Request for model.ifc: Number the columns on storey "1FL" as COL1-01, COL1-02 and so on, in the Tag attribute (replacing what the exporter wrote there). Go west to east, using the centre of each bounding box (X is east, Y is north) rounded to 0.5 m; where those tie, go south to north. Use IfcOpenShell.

First a look at what the model holds.

```python
import ifcopenshell
import ifcopenshell.util.element
import ifcopenshell.util.placement

model = ifcopenshell.open("model.ifc")
print(model.schema)
storey = next(s for s in model.by_type("IfcBuildingStorey") if s.Name == "1FL")
columns = [e for e in ifcopenshell.util.element.get_decomposition(storey) if e.is_a("IfcColumn")]
for e in sorted(columns, key=lambda e: e.id()):
    origin = ifcopenshell.util.placement.get_local_placement(e.ObjectPlacement)[:3, 3]
    print(e.id(), e.Tag, e.Name, origin.round(2) + 0.0, sep=" | ")
```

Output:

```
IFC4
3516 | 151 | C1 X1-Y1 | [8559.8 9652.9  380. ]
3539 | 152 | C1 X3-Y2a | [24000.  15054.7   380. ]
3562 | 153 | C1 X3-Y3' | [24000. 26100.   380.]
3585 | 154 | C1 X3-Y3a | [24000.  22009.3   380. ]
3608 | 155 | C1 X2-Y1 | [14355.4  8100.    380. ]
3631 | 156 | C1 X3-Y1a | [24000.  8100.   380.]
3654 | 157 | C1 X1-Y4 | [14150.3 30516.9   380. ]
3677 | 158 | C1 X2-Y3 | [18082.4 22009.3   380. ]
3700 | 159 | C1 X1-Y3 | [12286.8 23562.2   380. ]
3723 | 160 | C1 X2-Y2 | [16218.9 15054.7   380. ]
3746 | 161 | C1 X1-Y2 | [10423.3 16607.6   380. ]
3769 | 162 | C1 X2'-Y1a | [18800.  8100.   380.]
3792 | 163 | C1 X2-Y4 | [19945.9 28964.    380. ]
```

```python
import ifcopenshell
import ifcopenshell.geom
import ifcopenshell.util.element
import ifcopenshell.util.shape

model = ifcopenshell.open("model.ifc")
settings = ifcopenshell.geom.settings()
settings.set("use-world-coords", True)


def centre(element):
    shape = ifcopenshell.geom.create_shape(settings, element)
    return ifcopenshell.util.shape.get_bbox_centroid(shape.geometry)


storey = next(s for s in model.by_type("IfcBuildingStorey") if s.Name == "1FL")
columns = [e for e in ifcopenshell.util.element.get_decomposition(storey) if e.is_a("IfcColumn")]

# Insertion points can sit at a corner or the storey origin, so sort by the geometry (in metres).
centres = {e: centre(e) for e in columns}
columns.sort(key=lambda e: (round(centres[e][0] / 0.5), centres[e][1]))

for i, e in enumerate(columns, start=1):
    number = f"COL1-{i:02d}"
    e.Tag = number
    print(e.id(), number)

model.write("model_edited.ifc")
```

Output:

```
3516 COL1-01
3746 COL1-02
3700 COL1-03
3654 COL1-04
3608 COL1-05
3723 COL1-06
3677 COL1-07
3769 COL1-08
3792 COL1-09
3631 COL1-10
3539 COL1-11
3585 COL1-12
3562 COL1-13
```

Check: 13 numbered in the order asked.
